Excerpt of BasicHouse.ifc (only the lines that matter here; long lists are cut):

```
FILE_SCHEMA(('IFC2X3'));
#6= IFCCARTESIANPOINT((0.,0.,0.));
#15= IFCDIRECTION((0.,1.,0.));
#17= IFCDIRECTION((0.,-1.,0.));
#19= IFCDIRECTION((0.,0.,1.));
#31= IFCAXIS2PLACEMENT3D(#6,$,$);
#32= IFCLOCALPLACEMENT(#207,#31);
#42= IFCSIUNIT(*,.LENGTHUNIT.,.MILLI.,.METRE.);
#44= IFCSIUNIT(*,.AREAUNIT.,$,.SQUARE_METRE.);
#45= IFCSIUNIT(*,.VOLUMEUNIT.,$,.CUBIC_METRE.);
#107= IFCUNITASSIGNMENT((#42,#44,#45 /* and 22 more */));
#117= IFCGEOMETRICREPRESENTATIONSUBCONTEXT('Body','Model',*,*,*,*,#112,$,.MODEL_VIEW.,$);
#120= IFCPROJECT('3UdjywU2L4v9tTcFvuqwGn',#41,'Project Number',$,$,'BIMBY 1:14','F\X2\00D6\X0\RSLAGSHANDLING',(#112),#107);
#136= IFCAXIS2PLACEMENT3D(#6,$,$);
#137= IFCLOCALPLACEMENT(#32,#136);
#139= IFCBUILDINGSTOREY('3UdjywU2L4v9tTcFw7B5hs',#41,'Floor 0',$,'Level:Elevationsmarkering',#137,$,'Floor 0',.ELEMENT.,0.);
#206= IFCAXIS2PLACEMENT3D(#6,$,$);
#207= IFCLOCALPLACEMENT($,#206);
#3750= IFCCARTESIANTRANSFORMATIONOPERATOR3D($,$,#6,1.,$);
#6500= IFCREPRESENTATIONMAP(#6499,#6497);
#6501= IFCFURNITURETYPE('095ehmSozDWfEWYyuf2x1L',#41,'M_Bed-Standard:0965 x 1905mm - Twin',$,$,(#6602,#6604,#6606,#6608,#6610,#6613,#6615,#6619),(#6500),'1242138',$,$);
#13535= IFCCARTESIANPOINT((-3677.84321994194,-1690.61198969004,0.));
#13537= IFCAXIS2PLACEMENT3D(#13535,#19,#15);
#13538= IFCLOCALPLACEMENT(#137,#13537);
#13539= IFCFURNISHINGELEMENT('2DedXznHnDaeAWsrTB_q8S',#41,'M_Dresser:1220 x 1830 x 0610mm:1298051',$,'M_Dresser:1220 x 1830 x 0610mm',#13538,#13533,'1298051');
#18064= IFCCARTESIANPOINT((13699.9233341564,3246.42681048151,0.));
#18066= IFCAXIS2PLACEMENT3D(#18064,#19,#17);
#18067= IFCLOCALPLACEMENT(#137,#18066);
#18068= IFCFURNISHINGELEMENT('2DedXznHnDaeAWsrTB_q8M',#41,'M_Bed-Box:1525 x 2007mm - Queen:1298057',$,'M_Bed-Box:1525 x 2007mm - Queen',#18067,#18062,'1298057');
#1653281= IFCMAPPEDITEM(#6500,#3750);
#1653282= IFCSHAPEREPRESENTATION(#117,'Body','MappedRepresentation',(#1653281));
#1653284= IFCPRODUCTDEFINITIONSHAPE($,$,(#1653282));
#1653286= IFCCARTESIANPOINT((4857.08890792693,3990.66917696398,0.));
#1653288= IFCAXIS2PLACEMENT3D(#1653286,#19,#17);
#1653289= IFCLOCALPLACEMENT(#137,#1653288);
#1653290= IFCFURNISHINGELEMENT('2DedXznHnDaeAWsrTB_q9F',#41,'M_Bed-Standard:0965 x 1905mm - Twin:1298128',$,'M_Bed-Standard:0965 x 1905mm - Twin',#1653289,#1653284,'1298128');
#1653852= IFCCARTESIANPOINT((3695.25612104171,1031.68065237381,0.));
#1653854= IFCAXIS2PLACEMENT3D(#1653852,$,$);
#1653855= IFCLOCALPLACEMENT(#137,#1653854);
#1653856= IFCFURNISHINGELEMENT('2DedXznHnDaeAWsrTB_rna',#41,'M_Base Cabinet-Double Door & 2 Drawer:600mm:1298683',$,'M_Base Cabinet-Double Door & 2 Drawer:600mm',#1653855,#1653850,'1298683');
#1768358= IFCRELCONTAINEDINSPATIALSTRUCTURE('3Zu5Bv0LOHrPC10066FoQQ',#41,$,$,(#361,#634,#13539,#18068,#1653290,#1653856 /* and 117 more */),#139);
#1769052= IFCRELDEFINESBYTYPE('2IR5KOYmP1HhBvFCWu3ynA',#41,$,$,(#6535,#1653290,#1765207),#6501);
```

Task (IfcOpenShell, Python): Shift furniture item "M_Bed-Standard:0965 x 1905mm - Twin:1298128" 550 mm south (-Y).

```python
import ifcopenshell
import ifcopenshell.api.geometry
import ifcopenshell.util.placement
import ifcopenshell.util.unit

model = ifcopenshell.open("BasicHouse.ifc")
unit_scale = ifcopenshell.util.unit.calculate_unit_scale(model)

item = model.by_guid("2DedXznHnDaeAWsrTB_q9F")
matrix = ifcopenshell.util.placement.get_local_placement(item.ObjectPlacement)
matrix[1, 3] -= 0.55 / unit_scale
ifcopenshell.api.geometry.edit_object_placement(model, product=item, matrix=matrix, is_si=False)

print(ifcopenshell.util.placement.get_local_placement(item.ObjectPlacement).round(3) + 0.0)

model.write("BasicHouse_v2.ifc")
```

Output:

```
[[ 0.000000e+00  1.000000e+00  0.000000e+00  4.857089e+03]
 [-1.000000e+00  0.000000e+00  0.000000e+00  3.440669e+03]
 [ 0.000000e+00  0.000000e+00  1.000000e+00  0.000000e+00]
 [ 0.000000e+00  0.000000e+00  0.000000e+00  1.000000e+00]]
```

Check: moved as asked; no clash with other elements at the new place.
